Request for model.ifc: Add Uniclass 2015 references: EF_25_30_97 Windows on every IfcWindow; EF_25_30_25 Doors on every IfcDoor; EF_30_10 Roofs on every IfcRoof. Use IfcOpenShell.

First a look at what the model holds.

```python
import ifcopenshell

model = ifcopenshell.open("model.ifc")
print(model.schema)
print("classifications:", [c.Name for c in model.by_type("IfcClassification")])
for ifc_class in ("IfcDoor", "IfcRoof", "IfcStair", "IfcWall", "IfcWindow"):
    print(ifc_class, len(model.by_type(ifc_class)))
```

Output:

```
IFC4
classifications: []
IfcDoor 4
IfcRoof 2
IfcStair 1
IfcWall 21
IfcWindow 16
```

```python
import ifcopenshell
import ifcopenshell.api.classification

model = ifcopenshell.open("model.ifc")

system = ifcopenshell.api.classification.add_classification(model, classification="Uniclass 2015")

codes = {
    "IfcWindow": ("EF_25_30_97", "Windows"),
    "IfcDoor": ("EF_25_30_25", "Doors"),
    "IfcRoof": ("EF_30_10", "Roofs"),
}
for ifc_class, (code, name) in codes.items():
    products = model.by_type(ifc_class)
    ifcopenshell.api.classification.add_reference(
        model, products=products, classification=system, identification=code, name=name
    )
    print(code, len(products))

model.write("model_edited.ifc")
```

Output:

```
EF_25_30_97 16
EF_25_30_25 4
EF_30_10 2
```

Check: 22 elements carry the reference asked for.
